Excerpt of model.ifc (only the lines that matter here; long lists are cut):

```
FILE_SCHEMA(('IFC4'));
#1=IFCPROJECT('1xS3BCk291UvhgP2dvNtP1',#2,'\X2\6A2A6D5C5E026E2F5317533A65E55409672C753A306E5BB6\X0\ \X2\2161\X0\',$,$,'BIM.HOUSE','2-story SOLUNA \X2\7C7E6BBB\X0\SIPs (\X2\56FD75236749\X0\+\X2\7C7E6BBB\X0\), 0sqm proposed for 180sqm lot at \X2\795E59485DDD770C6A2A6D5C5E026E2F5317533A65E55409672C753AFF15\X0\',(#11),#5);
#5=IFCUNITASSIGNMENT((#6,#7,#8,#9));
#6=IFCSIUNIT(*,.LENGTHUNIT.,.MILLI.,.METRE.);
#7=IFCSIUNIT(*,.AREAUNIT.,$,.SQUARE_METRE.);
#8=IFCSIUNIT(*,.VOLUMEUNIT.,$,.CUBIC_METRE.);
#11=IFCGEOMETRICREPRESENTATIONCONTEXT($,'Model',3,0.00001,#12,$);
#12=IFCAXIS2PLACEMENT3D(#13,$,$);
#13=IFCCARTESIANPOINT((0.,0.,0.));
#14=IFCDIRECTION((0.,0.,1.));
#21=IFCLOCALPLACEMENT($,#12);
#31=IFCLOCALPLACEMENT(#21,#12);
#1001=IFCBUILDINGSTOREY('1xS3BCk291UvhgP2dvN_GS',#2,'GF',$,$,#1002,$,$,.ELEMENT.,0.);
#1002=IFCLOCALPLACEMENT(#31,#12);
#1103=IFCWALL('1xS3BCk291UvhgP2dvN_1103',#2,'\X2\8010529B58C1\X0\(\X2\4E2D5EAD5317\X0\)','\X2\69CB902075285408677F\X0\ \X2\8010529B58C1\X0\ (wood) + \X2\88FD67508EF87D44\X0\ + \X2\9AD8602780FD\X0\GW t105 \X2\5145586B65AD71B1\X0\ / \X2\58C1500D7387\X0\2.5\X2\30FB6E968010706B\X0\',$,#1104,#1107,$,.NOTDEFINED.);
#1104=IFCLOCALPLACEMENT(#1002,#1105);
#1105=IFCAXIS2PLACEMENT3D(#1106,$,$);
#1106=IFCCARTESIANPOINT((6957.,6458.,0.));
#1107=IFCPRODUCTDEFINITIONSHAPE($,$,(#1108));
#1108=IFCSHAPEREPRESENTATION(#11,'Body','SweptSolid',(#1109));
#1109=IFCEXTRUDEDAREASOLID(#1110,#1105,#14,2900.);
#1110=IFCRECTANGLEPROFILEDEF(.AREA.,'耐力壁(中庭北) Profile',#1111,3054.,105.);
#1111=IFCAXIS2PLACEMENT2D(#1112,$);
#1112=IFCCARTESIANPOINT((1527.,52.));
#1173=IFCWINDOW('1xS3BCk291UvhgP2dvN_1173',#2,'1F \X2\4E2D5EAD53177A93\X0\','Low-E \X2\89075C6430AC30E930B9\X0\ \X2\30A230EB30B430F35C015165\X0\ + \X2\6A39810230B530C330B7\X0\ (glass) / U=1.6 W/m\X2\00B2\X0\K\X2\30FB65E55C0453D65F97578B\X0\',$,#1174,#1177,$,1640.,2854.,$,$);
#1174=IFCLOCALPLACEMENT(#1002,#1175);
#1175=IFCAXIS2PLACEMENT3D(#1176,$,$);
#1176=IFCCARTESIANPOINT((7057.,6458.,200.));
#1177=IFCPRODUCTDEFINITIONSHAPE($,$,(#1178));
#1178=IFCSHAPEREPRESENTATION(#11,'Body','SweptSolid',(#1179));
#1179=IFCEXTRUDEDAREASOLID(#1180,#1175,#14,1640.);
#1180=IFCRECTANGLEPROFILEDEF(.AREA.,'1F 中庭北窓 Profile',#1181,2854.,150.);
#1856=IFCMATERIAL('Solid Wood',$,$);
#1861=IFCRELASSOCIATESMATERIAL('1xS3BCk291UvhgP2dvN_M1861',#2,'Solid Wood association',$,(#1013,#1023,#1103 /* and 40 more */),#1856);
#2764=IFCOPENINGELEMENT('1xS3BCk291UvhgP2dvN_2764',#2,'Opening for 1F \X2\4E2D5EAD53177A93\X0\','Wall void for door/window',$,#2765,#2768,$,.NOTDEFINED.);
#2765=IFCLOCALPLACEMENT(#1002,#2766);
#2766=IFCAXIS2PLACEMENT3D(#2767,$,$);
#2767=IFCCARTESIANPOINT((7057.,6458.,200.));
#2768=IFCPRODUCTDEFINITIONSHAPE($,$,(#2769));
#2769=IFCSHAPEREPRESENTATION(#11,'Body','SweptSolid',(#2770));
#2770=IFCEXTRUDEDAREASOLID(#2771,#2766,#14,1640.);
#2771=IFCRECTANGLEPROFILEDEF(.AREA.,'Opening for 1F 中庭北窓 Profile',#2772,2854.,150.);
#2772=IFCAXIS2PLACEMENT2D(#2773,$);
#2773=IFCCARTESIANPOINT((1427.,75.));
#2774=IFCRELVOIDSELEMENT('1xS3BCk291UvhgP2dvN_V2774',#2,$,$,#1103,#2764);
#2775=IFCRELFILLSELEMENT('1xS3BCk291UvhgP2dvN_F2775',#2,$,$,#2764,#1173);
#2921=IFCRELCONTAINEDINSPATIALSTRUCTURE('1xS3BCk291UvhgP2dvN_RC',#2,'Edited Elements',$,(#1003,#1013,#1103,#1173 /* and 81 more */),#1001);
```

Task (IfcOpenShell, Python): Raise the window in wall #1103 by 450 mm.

```python
import numpy as np
import ifcopenshell
import ifcopenshell.api.geometry
import ifcopenshell.util.placement
import ifcopenshell.util.unit

model = ifcopenshell.open("model.ifc")
unit_scale = ifcopenshell.util.unit.calculate_unit_scale(model)

window = model.by_guid("1xS3BCk291UvhgP2dvN_1173")
opening = window.FillsVoids[0].RelatingOpeningElement
dz = 450.0

shift = np.array([0.0, 0.0, dz])
# The window is not placed relative to its opening, so move both.
for product in (opening, window):
    matrix = ifcopenshell.util.placement.get_local_placement(product.ObjectPlacement)
    matrix[:3, 3] += shift
    ifcopenshell.api.geometry.edit_object_placement(model, product=product, matrix=matrix, is_si=False)

print(f"moved by {dz * unit_scale:+.3f} m")

model.write("model_v2.ifc")
```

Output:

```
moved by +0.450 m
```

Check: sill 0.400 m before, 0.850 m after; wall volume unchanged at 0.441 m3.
